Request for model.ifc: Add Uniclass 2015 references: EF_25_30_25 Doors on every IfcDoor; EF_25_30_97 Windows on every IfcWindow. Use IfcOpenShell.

First a look at what the model holds.

```python
import ifcopenshell

model = ifcopenshell.open("model.ifc")
print(model.schema)
print("classifications:", [c.Name for c in model.by_type("IfcClassification")])
for ifc_class in ("IfcDoor", "IfcRoof", "IfcStair", "IfcWall", "IfcWindow"):
    print(ifc_class, len(model.by_type(ifc_class)))
```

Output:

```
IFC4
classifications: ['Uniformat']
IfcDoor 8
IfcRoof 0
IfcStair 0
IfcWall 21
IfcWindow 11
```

```python
import ifcopenshell
import ifcopenshell.api.classification

model = ifcopenshell.open("model.ifc")

system = ifcopenshell.api.classification.add_classification(model, classification="Uniclass 2015")

codes = {
    "IfcDoor": ("EF_25_30_25", "Doors"),
    "IfcWindow": ("EF_25_30_97", "Windows"),
}
for ifc_class, (code, name) in codes.items():
    products = model.by_type(ifc_class)
    ifcopenshell.api.classification.add_reference(
        model, products=products, classification=system, identification=code, name=name
    )
    print(code, len(products))

model.write("model-out.ifc")
```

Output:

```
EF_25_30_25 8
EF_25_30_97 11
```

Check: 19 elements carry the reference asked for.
